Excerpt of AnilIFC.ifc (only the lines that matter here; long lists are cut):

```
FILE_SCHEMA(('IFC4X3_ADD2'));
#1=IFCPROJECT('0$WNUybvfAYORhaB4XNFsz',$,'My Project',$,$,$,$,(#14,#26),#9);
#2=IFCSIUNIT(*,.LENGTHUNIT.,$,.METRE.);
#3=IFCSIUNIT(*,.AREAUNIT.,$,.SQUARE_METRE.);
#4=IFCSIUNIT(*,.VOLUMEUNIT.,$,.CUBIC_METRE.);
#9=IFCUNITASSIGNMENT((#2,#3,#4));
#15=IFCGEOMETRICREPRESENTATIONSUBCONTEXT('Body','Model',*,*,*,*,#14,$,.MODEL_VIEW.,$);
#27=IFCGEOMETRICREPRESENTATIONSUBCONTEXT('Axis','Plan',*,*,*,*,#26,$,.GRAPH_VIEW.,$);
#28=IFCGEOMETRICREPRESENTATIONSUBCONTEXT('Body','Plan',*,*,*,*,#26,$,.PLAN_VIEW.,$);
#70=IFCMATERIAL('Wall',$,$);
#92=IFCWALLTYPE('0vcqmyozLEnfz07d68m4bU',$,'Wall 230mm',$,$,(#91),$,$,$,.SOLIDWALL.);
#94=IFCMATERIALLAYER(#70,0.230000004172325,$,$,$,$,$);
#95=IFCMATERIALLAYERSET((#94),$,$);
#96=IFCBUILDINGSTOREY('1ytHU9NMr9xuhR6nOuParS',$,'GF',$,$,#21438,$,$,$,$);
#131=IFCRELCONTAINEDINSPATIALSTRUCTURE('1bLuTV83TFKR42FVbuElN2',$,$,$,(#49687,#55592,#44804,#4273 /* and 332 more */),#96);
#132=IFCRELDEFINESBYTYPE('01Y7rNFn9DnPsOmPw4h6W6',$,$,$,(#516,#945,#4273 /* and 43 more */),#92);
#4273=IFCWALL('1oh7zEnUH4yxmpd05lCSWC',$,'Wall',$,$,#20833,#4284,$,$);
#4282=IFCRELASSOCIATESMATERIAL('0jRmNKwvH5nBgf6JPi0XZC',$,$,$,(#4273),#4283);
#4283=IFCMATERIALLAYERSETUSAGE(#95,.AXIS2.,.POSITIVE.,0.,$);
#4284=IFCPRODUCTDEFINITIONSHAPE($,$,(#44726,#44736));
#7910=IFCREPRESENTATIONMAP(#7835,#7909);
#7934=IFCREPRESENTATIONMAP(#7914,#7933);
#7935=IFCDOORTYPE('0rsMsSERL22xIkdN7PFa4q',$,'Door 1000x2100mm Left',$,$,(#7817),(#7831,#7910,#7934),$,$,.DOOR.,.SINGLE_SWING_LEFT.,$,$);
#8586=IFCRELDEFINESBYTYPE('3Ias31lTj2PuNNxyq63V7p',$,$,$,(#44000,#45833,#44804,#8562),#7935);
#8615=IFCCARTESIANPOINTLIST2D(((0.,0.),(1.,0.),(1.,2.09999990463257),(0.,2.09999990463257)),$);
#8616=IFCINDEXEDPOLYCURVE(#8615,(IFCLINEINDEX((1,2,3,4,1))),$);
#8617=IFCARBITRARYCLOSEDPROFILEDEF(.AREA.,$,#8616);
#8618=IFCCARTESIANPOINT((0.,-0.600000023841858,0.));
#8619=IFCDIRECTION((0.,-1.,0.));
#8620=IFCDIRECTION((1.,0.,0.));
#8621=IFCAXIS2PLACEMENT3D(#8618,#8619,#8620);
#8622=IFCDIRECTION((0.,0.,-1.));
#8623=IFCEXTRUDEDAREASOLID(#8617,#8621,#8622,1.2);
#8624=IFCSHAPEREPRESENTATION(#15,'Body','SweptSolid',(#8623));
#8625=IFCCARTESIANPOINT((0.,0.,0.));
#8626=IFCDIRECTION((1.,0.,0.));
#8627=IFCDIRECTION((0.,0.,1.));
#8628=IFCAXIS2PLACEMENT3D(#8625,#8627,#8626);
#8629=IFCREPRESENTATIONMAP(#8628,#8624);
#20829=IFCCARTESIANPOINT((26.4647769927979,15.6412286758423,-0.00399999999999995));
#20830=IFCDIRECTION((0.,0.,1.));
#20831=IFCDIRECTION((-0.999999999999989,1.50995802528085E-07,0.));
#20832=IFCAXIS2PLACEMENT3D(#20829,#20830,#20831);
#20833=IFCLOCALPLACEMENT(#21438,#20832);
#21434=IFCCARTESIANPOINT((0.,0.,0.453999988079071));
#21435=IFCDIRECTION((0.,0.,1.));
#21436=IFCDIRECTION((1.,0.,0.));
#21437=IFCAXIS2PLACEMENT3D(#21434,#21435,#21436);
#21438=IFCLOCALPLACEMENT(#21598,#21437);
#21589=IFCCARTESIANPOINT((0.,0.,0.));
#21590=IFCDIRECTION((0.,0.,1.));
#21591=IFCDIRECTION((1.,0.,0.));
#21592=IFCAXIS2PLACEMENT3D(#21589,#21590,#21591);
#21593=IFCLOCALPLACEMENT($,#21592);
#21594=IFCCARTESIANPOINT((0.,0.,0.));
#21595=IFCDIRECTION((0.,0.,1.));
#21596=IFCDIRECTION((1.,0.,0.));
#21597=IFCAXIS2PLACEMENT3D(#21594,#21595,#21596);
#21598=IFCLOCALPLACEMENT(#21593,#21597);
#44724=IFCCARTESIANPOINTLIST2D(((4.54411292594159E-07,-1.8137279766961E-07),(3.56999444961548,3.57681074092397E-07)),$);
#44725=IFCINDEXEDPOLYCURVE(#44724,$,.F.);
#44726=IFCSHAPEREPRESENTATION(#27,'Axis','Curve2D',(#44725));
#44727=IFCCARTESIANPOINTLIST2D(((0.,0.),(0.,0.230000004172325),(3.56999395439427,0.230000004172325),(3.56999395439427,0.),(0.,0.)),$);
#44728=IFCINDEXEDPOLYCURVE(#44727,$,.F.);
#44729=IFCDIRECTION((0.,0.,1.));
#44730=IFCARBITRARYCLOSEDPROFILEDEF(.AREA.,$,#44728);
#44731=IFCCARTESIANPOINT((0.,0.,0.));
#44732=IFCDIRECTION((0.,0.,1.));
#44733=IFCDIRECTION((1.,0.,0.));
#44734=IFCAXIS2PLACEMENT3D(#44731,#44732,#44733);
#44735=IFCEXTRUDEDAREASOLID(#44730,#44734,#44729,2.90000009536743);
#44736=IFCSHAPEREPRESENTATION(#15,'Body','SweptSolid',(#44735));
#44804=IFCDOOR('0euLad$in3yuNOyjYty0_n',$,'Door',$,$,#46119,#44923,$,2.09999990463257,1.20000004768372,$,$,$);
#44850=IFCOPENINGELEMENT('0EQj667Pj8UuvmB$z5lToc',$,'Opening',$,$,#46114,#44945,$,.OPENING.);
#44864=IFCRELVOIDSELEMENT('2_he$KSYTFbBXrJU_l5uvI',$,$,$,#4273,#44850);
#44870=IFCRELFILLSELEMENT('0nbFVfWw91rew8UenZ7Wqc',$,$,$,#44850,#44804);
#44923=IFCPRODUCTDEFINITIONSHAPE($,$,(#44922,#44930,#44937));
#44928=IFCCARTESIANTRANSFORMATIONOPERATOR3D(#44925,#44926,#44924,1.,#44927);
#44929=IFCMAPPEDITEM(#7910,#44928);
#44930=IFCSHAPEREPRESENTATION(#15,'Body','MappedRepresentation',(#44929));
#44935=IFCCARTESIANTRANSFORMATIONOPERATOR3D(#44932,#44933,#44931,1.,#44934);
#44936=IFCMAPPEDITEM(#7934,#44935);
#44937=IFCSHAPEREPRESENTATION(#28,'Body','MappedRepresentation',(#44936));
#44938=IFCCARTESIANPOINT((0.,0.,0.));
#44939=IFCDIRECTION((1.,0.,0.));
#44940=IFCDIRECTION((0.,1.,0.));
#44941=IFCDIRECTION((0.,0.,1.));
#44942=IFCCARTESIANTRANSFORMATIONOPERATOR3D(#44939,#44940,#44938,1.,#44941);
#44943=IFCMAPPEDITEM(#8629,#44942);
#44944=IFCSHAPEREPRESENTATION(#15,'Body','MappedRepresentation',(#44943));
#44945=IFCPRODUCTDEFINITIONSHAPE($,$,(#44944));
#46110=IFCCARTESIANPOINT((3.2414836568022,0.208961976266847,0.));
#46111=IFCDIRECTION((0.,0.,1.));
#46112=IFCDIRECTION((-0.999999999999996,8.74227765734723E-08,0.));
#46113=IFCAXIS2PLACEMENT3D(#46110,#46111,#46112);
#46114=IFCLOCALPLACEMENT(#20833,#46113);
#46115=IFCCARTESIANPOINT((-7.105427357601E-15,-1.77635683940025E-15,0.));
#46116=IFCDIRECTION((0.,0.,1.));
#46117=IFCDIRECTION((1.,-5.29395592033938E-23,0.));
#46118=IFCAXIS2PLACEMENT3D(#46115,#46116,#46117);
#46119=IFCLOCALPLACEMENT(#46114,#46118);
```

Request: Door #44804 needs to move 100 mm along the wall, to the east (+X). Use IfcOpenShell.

```python
import ifcopenshell
import ifcopenshell.api.geometry
import ifcopenshell.util.placement
import ifcopenshell.util.unit

model = ifcopenshell.open("AnilIFC.ifc")
unit_scale = ifcopenshell.util.unit.calculate_unit_scale(model)

door = model.by_guid("0euLad$in3yuNOyjYty0_n")
opening = door.FillsVoids[0].RelatingOpeningElement
wall = opening.VoidsElements[0].RelatingBuildingElement

wall_matrix = ifcopenshell.util.placement.get_local_placement(wall.ObjectPlacement)
shift = wall_matrix[:3, 0] * -0.1 / unit_scale
before = ifcopenshell.util.placement.get_local_placement(door.ObjectPlacement)[:3, 3].copy()

# The door is placed relative to its opening, so it follows when the opening moves.
matrix = ifcopenshell.util.placement.get_local_placement(opening.ObjectPlacement)
matrix[:3, 3] += shift
ifcopenshell.api.geometry.edit_object_placement(
    model, product=opening, matrix=matrix, is_si=False, should_transform_children=True
)

after = ifcopenshell.util.placement.get_local_placement(door.ObjectPlacement)[:3, 3]
print("door moved by", (after - before).round(3) + 0.0)

model.write("AnilIFC-out.ifc")
```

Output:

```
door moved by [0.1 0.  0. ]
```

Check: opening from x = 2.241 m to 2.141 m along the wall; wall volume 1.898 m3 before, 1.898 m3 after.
